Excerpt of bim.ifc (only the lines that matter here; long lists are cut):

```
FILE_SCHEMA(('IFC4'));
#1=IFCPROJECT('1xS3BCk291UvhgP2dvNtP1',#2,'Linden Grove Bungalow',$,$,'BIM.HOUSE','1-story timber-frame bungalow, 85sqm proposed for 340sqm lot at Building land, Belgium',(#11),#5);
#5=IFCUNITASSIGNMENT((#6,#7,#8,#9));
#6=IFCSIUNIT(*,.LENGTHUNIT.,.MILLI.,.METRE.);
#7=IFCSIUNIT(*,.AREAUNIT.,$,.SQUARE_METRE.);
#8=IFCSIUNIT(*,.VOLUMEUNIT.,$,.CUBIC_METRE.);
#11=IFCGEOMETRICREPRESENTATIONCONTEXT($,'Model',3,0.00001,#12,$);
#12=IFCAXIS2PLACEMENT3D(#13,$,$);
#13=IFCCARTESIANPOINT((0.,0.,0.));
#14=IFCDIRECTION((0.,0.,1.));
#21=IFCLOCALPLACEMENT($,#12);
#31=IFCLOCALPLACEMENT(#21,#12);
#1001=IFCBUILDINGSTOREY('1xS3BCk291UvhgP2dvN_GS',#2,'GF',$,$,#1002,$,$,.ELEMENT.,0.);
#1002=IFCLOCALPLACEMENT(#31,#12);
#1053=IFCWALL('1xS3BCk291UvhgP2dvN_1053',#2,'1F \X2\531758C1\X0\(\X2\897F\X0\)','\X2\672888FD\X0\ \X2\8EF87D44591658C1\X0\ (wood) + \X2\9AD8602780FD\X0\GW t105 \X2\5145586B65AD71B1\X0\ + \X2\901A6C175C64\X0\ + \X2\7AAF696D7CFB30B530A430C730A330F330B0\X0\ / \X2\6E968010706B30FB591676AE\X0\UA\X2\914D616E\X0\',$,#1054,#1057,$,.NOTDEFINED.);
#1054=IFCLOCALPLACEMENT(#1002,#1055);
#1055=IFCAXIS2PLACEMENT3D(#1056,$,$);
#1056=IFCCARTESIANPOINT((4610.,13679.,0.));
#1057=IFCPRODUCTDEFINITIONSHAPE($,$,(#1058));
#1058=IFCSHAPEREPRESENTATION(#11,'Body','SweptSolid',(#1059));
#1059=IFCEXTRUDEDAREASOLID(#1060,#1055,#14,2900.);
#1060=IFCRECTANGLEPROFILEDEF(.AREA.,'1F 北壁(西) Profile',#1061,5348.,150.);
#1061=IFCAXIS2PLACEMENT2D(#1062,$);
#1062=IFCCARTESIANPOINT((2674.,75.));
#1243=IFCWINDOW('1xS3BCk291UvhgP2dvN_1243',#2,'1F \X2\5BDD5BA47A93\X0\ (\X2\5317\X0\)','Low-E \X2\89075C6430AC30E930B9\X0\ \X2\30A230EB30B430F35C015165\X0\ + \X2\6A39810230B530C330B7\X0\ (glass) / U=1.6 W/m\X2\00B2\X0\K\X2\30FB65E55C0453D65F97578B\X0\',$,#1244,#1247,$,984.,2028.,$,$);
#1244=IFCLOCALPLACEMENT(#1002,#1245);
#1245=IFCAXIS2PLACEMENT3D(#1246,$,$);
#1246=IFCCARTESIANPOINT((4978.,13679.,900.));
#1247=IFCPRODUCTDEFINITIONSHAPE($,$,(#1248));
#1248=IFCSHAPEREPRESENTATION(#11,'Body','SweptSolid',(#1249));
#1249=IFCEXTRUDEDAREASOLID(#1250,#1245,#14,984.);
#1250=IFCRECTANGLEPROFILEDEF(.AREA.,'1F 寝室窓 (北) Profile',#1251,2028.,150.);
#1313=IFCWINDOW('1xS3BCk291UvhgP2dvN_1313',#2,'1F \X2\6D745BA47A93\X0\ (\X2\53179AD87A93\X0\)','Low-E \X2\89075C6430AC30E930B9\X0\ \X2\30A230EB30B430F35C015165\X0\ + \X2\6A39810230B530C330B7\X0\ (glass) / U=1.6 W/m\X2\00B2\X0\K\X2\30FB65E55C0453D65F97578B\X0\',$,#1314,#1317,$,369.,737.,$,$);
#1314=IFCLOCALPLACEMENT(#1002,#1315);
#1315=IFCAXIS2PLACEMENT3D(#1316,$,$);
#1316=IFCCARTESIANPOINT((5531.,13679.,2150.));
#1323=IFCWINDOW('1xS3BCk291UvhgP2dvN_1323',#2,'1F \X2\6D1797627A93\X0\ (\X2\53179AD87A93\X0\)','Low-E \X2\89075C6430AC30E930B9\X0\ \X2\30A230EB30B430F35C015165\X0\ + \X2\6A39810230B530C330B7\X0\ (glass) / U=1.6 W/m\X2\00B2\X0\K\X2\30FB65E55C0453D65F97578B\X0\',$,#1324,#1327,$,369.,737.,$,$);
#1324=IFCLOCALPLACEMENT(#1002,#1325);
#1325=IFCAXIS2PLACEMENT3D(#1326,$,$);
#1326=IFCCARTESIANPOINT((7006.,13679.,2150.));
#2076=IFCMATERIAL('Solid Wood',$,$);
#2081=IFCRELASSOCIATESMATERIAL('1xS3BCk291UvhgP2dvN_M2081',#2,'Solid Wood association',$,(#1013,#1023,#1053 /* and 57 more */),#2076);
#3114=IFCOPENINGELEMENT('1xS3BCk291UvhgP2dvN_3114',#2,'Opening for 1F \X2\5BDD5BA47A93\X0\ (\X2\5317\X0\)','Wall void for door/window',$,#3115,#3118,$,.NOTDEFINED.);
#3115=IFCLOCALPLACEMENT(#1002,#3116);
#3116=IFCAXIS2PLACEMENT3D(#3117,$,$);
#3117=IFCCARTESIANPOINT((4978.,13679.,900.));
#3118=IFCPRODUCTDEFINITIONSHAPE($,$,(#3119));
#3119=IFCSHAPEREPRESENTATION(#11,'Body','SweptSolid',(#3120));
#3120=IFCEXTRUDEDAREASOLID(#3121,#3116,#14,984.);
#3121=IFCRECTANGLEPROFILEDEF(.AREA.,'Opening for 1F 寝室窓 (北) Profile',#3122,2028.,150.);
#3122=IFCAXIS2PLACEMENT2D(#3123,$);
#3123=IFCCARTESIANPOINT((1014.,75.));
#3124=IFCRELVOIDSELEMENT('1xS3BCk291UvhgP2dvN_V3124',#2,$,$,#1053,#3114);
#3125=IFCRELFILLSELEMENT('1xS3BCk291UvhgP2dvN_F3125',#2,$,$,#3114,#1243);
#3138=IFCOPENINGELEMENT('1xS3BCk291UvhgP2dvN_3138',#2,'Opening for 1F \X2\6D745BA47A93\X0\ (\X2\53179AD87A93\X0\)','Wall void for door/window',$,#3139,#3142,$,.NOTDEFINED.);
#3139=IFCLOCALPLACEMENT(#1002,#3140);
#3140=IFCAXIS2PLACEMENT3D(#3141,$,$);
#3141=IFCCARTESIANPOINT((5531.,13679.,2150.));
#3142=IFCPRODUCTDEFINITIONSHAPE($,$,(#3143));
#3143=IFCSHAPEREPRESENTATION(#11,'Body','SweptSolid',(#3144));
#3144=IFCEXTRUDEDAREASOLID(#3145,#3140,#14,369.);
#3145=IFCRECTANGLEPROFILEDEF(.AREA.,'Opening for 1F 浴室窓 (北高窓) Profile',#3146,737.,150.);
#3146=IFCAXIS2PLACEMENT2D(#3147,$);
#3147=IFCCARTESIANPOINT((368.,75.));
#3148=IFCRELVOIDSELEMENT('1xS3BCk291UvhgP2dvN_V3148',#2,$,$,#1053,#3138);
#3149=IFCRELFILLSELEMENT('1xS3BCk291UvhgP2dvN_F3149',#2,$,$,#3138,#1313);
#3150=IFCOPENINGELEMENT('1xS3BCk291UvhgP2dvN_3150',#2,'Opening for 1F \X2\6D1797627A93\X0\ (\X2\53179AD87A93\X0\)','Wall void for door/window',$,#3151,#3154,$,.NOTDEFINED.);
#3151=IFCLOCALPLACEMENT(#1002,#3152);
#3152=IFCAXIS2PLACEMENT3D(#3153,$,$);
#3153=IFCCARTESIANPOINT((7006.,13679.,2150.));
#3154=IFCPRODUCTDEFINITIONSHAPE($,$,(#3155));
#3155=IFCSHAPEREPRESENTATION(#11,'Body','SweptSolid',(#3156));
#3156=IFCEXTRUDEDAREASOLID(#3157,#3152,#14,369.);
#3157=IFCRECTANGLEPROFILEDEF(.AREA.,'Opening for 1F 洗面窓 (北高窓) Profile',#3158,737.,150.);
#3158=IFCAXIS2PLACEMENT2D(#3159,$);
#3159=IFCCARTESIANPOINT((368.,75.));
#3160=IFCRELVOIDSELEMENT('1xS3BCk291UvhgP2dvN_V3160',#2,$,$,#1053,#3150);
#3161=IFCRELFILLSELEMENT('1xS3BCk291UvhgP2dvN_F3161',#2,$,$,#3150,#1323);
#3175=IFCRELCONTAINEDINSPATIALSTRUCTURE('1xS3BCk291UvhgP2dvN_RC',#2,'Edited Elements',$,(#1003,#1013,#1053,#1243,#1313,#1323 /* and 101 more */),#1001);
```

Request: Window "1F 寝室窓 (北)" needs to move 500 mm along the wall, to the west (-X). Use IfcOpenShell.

```python
import ifcopenshell
import ifcopenshell.api.geometry
import ifcopenshell.util.placement

model = ifcopenshell.open("bim.ifc")

window = model.by_guid("1xS3BCk291UvhgP2dvN_1243")
opening = window.FillsVoids[0].RelatingOpeningElement
wall = opening.VoidsElements[0].RelatingBuildingElement

wall_matrix = ifcopenshell.util.placement.get_local_placement(wall.ObjectPlacement)
shift = wall_matrix[:3, 0] * -500.0
before = ifcopenshell.util.placement.get_local_placement(window.ObjectPlacement)[:3, 3].copy()

# The window is not placed relative to its opening, so move both.
for product in (opening, window):
    matrix = ifcopenshell.util.placement.get_local_placement(product.ObjectPlacement)
    matrix[:3, 3] += shift
    ifcopenshell.api.geometry.edit_object_placement(model, product=product, matrix=matrix, is_si=False)

after = ifcopenshell.util.placement.get_local_placement(window.ObjectPlacement)[:3, 3]
print("window moved by", (after - before).round(3) + 0.0)

model.write("bim_v2.ifc")
```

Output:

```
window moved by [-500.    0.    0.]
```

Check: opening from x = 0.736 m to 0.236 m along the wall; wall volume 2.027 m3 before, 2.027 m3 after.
